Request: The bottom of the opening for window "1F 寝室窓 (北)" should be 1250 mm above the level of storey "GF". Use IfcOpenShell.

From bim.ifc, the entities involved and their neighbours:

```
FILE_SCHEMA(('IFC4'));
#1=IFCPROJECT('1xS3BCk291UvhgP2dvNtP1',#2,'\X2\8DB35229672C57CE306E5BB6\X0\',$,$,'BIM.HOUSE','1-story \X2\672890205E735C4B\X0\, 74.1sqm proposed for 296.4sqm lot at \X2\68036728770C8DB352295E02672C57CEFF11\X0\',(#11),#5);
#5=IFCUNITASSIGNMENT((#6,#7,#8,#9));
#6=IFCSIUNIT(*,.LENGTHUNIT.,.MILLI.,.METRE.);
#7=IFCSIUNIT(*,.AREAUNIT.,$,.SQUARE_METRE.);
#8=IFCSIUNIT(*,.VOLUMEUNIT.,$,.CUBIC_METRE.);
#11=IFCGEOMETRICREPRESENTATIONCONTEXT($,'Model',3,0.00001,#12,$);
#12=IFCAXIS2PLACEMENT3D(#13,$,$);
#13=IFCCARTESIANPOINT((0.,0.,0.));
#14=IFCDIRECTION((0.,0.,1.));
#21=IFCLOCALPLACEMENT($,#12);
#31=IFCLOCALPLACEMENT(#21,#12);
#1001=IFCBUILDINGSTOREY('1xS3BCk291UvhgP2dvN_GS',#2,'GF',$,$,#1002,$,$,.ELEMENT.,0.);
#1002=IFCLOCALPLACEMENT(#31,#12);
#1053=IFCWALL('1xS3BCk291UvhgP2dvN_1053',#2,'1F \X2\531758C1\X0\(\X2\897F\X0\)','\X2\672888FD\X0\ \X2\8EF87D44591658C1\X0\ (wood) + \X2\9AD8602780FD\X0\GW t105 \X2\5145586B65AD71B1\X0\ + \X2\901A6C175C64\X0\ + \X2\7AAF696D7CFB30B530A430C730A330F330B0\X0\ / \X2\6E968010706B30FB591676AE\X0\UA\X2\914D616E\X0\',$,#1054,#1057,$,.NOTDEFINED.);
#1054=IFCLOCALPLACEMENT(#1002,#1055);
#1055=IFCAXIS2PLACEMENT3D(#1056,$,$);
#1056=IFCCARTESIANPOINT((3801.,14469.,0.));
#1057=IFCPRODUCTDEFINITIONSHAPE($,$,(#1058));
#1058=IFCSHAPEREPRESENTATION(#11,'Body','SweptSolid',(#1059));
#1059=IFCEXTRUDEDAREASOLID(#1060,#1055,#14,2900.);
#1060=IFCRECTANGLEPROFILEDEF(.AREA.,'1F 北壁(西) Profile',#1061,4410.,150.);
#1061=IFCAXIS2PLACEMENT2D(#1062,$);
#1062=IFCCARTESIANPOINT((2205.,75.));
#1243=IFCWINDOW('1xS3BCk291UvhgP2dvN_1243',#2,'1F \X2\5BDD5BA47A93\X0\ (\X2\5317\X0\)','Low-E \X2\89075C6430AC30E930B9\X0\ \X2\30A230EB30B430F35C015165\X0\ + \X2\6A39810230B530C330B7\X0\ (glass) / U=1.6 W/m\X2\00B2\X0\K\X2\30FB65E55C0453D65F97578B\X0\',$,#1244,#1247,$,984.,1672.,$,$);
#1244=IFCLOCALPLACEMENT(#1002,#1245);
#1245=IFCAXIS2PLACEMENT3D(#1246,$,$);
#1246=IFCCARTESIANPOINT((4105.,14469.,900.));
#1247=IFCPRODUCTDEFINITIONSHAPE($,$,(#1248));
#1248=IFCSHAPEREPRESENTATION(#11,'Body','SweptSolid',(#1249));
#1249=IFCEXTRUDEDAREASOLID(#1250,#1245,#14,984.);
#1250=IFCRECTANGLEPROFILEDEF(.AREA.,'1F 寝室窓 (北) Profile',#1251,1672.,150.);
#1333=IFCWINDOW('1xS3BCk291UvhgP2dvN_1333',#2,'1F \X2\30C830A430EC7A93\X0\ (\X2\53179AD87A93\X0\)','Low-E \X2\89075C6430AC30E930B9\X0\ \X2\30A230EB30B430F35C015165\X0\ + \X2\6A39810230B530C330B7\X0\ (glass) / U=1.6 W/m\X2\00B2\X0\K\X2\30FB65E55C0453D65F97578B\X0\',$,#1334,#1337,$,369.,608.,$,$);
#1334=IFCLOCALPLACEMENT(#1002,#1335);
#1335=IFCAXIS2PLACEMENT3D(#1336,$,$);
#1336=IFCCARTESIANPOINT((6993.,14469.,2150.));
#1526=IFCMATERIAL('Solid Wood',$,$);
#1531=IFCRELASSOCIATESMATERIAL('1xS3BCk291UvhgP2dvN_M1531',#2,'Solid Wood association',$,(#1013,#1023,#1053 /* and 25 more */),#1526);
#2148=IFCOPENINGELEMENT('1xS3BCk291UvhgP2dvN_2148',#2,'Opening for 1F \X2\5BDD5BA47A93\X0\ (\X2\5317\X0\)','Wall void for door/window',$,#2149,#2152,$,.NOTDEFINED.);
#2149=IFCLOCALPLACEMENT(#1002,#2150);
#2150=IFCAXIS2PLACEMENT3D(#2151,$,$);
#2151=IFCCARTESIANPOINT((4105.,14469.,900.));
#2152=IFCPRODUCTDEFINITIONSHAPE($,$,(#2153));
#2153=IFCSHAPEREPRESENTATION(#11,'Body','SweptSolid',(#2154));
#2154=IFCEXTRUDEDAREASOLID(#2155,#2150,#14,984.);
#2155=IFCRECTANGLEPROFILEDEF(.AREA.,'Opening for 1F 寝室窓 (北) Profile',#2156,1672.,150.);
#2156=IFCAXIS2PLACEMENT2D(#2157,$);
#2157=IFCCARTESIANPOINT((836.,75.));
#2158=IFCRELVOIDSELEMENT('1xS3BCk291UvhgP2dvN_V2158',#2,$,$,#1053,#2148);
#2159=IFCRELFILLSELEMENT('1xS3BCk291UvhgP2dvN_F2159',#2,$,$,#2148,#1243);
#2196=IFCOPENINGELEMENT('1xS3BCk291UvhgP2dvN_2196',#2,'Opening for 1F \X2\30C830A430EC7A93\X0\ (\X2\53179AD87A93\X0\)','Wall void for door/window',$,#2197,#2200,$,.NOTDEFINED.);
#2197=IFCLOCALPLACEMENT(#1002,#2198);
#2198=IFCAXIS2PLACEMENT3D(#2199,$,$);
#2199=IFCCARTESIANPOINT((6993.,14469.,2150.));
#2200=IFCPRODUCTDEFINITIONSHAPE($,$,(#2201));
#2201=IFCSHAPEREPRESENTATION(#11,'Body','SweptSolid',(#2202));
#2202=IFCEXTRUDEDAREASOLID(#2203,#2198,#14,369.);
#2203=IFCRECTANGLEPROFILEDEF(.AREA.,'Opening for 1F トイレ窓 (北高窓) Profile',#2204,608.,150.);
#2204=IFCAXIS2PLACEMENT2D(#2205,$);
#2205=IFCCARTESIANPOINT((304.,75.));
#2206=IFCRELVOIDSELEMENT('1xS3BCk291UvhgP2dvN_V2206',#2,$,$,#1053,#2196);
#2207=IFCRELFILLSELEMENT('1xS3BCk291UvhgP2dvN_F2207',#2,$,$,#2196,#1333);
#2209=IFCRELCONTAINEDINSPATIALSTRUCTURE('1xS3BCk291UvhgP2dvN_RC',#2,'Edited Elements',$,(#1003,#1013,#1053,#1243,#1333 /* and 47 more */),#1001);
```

```python
import numpy as np
import ifcopenshell
import ifcopenshell.api.geometry
import ifcopenshell.geom
import ifcopenshell.util.element
import ifcopenshell.util.placement
import ifcopenshell.util.shape
import ifcopenshell.util.unit

model = ifcopenshell.open("bim.ifc")
unit_scale = ifcopenshell.util.unit.calculate_unit_scale(model)

window = model.by_id(1243)
opening = window.FillsVoids[0].RelatingOpeningElement
storey = ifcopenshell.util.element.get_container(window, ifc_class="IfcBuildingStorey")
level = ifcopenshell.util.placement.get_local_placement(storey.ObjectPlacement)[2, 3]

# The opening's origin need not be at the sill, so measure its lowest point.
shape = ifcopenshell.geom.create_shape(ifcopenshell.geom.settings(), opening)
bottom = ifcopenshell.util.shape.get_shape_bottom_elevation(shape, shape.geometry) / unit_scale
dz = level + 1.25 / unit_scale - bottom

shift = np.array([0.0, 0.0, dz])
# The window is not placed relative to its opening, so move both.
for product in (opening, window):
    matrix = ifcopenshell.util.placement.get_local_placement(product.ObjectPlacement)
    matrix[:3, 3] += shift
    ifcopenshell.api.geometry.edit_object_placement(model, product=product, matrix=matrix, is_si=False)

print(f"moved by {dz * unit_scale:+.3f} m")

model.write("bim_v2.ifc")
```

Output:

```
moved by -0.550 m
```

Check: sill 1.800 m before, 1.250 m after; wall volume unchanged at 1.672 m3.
